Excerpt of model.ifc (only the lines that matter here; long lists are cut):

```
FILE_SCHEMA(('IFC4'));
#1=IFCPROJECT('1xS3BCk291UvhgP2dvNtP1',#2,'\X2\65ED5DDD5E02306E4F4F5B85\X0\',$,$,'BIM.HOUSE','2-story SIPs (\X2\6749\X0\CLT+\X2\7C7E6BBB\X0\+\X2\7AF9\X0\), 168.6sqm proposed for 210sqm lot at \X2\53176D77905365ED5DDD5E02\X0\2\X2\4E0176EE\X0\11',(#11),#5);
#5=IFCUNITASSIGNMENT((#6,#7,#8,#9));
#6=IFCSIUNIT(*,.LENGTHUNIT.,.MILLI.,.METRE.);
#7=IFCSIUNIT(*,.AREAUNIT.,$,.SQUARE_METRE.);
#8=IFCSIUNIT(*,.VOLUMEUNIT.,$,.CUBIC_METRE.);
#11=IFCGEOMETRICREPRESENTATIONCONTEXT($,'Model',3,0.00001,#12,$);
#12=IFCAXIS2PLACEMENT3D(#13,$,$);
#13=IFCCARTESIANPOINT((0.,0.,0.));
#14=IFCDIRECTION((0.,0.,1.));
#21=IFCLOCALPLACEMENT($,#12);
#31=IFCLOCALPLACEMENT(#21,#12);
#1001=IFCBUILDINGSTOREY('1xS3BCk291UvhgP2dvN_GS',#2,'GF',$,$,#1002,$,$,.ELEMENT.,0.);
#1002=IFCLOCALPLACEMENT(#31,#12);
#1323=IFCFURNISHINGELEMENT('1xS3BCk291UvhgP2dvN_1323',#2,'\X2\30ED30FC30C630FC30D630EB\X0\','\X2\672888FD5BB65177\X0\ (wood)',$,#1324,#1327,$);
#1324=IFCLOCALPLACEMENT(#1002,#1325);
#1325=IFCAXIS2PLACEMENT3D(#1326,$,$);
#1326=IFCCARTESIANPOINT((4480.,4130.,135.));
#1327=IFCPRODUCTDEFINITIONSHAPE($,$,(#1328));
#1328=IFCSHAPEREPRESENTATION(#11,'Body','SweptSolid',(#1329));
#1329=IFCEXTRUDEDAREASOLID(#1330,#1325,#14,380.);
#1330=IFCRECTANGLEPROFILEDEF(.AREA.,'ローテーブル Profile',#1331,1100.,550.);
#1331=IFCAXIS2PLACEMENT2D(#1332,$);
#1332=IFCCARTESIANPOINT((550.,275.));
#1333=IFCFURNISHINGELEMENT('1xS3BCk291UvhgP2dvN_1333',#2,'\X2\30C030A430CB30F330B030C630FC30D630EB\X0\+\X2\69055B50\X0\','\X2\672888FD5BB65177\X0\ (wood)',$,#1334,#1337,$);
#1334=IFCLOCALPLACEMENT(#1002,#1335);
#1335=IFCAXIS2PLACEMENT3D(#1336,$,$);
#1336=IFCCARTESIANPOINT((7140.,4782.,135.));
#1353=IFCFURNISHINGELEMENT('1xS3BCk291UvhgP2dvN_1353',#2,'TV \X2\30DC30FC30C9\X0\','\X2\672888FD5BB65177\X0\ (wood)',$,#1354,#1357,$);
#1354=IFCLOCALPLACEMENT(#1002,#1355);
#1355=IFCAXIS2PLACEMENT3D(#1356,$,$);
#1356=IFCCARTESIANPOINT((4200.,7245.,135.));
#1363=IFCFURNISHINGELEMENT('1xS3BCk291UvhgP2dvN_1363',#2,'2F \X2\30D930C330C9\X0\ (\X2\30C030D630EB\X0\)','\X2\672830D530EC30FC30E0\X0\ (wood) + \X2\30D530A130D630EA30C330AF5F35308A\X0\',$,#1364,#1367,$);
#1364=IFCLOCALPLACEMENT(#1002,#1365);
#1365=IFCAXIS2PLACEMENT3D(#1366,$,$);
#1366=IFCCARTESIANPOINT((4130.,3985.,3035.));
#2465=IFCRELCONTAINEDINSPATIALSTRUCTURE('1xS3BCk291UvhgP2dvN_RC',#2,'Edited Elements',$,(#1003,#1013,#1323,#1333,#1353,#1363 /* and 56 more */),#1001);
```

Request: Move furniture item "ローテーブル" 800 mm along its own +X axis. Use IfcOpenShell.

```python
import ifcopenshell
import ifcopenshell.api.geometry
import ifcopenshell.util.placement

model = ifcopenshell.open("model.ifc")

item = model.by_guid("1xS3BCk291UvhgP2dvN_1323")
matrix = ifcopenshell.util.placement.get_local_placement(item.ObjectPlacement)
matrix[:3, 3] += matrix[:3, 0] * 800.0
ifcopenshell.api.geometry.edit_object_placement(model, product=item, matrix=matrix, is_si=False)

print(ifcopenshell.util.placement.get_local_placement(item.ObjectPlacement).round(3) + 0.0)

model.write("model_v2.ifc")
```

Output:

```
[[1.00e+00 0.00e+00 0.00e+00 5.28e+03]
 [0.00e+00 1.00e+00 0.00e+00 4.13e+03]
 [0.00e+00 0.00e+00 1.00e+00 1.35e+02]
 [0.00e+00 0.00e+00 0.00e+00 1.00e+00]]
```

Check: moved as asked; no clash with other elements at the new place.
